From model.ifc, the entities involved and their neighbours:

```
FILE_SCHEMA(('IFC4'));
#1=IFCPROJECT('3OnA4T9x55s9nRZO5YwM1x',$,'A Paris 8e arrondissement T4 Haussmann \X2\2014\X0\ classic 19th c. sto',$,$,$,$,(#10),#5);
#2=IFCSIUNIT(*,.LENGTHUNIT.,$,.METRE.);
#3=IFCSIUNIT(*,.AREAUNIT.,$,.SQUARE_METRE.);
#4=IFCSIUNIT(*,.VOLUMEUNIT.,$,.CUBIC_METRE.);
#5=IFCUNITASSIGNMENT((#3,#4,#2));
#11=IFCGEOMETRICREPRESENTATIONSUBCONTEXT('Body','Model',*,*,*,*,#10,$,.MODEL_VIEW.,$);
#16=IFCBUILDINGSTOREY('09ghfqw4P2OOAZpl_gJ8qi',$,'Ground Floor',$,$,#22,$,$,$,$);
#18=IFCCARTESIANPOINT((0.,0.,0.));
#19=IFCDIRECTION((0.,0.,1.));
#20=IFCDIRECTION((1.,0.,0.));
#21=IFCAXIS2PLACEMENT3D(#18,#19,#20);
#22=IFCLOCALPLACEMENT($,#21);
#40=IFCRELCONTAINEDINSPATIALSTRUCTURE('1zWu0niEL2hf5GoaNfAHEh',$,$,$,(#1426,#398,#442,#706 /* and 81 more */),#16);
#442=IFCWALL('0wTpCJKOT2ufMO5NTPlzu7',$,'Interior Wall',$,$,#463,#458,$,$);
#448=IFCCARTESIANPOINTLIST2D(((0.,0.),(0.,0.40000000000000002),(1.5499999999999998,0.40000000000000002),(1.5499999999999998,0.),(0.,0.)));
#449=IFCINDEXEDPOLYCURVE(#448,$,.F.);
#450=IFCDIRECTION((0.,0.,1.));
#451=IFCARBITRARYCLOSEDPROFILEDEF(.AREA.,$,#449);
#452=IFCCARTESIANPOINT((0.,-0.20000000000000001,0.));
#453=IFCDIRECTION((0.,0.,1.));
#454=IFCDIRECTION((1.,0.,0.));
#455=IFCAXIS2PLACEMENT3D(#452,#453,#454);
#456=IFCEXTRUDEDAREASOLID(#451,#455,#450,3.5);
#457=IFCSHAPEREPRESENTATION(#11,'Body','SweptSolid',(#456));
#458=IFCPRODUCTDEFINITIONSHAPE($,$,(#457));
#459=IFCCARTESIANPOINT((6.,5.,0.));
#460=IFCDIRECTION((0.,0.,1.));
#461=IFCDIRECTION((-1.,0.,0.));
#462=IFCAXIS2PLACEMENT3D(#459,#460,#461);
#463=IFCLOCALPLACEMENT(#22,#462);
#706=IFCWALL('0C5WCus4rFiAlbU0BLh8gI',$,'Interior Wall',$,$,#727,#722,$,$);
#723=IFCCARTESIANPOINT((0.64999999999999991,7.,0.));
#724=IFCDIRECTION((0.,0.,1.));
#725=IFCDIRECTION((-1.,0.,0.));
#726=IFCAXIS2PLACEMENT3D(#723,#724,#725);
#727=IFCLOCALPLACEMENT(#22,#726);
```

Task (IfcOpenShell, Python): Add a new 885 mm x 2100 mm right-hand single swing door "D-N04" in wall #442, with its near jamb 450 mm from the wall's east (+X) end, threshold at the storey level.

```python
import numpy as np
import ifcopenshell
import ifcopenshell.api.feature
import ifcopenshell.api.geometry
import ifcopenshell.api.root
import ifcopenshell.api.spatial
import ifcopenshell.geom
import ifcopenshell.util.element
import ifcopenshell.util.placement
import ifcopenshell.util.representation
import ifcopenshell.util.shape
import ifcopenshell.util.unit

model = ifcopenshell.open("model.ifc")
unit_scale = ifcopenshell.util.unit.calculate_unit_scale(model)
settings = ifcopenshell.geom.settings()


def volume(element):
    """Net volume in cubic metres, openings subtracted."""
    shape = ifcopenshell.geom.create_shape(settings, element)
    return ifcopenshell.util.shape.get_volume(shape.geometry)


wall = model.by_guid("0wTpCJKOT2ufMO5NTPlzu7")
storey = ifcopenshell.util.element.get_container(wall, ifc_class="IfcBuildingStorey")
context = ifcopenshell.util.representation.get_context(model, "Model", "Body", "MODEL_VIEW")
before = volume(wall)

width, height, from_end, sill = 0.885, 2.1, 0.45, 0.0  # metres

# The wall runs along its own X axis, and the end named is its -X end.
wall_shape = ifcopenshell.geom.create_shape(settings, wall)
x, y, z = ifcopenshell.util.shape.get_vertices(wall_shape.geometry).T
start = x.min() + from_end
face, thickness = float(y.min()), float(y.max() - y.min())
wall_matrix = ifcopenshell.util.placement.get_local_placement(wall.ObjectPlacement)
level = ifcopenshell.util.placement.get_local_placement(storey.ObjectPlacement)[2, 3]


def in_wall(x, y):
    """Placement at x, y metres in the wall's axes, at sill height."""
    matrix = wall_matrix.copy()
    matrix[:, 3] = wall_matrix @ np.array([x / unit_scale, y / unit_scale, 0.0, 1.0])
    matrix[2, 3] = level + sill / unit_scale
    return matrix


# Opening: a box that overshoots both wall faces by 50 mm.
opening = ifcopenshell.api.root.create_entity(model, ifc_class="IfcOpeningElement", predefined_type="OPENING")
box = ifcopenshell.api.geometry.add_wall_representation(
    model, context=context, length=width, height=height, thickness=thickness + 0.1
)
ifcopenshell.api.geometry.assign_representation(model, product=opening, representation=box)
ifcopenshell.api.geometry.edit_object_placement(model, product=opening, matrix=in_wall(start, face - 0.05), is_si=False)
ifcopenshell.api.feature.add_feature(model, feature=opening, element=wall)

door = ifcopenshell.api.root.create_entity(model, ifc_class="IfcDoor", name="D-N04", predefined_type="DOOR")
door.OverallWidth, door.OverallHeight = width / unit_scale, height / unit_scale
door.OperationType = "SINGLE_SWING_RIGHT"
body = ifcopenshell.api.geometry.add_door_representation(
    model,
    context=context,
    overall_width=door.OverallWidth,
    overall_height=door.OverallHeight,
    operation_type="SINGLE_SWING_RIGHT",
    lining_properties={"LiningDepth": thickness / unit_scale, "ThresholdDepth": thickness / unit_scale},
)
ifcopenshell.api.geometry.assign_representation(model, product=door, representation=body)
ifcopenshell.api.spatial.assign_container(model, products=[door], relating_structure=storey)
ifcopenshell.api.feature.add_filling(model, opening=opening, element=door)

# The lining spans the wall, so the door starts at the wall face.
ifcopenshell.api.geometry.edit_object_placement(model, product=door, matrix=in_wall(start, face), is_si=False)

after = volume(wall)

print(f"wall volume {before:.3f} -> {after:.3f} m3")

model.write("model_edited.ifc")
```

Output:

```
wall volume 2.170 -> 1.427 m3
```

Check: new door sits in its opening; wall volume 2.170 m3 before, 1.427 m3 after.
